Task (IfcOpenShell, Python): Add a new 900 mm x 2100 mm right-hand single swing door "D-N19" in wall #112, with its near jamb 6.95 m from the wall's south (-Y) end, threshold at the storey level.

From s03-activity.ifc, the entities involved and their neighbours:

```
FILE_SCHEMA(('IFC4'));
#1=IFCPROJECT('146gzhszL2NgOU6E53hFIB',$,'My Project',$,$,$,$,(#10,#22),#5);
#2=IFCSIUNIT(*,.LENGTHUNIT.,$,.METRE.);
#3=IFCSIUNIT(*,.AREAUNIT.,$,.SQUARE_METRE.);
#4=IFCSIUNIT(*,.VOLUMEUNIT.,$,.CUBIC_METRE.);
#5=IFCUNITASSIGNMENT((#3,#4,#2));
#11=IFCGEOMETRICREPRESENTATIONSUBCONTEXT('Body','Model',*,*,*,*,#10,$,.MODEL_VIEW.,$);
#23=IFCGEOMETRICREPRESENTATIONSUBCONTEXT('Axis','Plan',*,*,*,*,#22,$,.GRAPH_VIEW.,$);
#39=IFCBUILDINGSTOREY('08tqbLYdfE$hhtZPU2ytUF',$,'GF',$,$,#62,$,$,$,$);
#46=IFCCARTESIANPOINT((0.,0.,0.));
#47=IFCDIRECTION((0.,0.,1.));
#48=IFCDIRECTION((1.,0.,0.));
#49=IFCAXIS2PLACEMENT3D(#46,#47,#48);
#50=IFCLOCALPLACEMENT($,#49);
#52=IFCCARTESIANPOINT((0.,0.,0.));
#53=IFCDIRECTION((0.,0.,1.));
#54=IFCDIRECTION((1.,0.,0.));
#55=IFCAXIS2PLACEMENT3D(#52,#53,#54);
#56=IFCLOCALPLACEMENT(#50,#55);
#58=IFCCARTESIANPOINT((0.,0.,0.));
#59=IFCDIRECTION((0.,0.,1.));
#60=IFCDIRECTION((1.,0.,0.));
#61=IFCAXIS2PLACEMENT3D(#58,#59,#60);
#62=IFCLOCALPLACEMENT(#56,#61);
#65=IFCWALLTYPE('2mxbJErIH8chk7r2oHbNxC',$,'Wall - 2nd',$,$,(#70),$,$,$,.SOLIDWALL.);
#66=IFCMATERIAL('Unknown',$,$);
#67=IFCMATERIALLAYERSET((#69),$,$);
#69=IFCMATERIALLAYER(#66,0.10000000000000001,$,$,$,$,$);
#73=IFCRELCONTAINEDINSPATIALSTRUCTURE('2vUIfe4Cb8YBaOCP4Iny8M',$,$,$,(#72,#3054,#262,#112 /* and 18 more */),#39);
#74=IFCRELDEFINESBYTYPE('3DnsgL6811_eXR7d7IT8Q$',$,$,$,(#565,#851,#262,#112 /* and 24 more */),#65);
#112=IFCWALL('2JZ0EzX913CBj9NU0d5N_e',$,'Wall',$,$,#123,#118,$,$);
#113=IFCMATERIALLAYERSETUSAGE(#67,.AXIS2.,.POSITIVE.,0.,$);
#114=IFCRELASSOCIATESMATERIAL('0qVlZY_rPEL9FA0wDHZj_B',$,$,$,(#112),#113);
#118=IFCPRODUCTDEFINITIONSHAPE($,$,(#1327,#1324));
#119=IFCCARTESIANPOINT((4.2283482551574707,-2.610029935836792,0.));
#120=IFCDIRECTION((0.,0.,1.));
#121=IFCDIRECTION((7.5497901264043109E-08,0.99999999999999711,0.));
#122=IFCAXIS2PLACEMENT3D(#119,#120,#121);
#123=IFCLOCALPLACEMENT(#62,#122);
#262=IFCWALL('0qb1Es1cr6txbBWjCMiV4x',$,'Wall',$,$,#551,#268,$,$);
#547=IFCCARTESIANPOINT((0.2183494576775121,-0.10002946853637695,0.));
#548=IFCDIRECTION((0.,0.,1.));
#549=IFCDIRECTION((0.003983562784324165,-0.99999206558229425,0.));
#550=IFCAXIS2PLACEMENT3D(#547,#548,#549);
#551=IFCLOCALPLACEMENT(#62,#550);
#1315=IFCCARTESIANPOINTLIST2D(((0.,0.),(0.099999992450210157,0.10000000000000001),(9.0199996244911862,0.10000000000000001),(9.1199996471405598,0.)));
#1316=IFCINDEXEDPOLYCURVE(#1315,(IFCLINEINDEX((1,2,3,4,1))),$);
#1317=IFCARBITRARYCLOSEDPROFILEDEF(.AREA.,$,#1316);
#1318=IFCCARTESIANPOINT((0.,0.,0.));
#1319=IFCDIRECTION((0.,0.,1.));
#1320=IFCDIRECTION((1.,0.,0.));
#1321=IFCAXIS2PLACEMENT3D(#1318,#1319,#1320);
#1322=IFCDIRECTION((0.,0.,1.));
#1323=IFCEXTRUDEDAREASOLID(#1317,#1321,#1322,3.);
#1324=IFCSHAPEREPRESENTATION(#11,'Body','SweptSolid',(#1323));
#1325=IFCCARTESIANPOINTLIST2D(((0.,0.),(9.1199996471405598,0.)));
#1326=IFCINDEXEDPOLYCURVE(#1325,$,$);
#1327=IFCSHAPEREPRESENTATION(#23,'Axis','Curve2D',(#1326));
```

```python
import numpy as np
import ifcopenshell
import ifcopenshell.api.feature
import ifcopenshell.api.geometry
import ifcopenshell.api.root
import ifcopenshell.api.spatial
import ifcopenshell.geom
import ifcopenshell.util.element
import ifcopenshell.util.placement
import ifcopenshell.util.representation
import ifcopenshell.util.shape
import ifcopenshell.util.unit

model = ifcopenshell.open("s03-activity.ifc")
unit_scale = ifcopenshell.util.unit.calculate_unit_scale(model)
settings = ifcopenshell.geom.settings()


def volume(element):
    """Net volume in cubic metres, openings subtracted."""
    shape = ifcopenshell.geom.create_shape(settings, element)
    return ifcopenshell.util.shape.get_volume(shape.geometry)


wall = model.by_guid("2JZ0EzX913CBj9NU0d5N_e")
storey = ifcopenshell.util.element.get_container(wall, ifc_class="IfcBuildingStorey")
context = ifcopenshell.util.representation.get_context(model, "Model", "Body", "MODEL_VIEW")
before = volume(wall)

width, height, from_end, sill = 0.9, 2.1, 6.95, 0.0  # metres

# The wall runs along its own X axis, and the end named is its -X end.
wall_shape = ifcopenshell.geom.create_shape(settings, wall)
x, y, z = ifcopenshell.util.shape.get_vertices(wall_shape.geometry).T
start = x.min() + from_end
face, thickness = float(y.min()), float(y.max() - y.min())
wall_matrix = ifcopenshell.util.placement.get_local_placement(wall.ObjectPlacement)
level = ifcopenshell.util.placement.get_local_placement(storey.ObjectPlacement)[2, 3]


def in_wall(x, y):
    """Placement at x, y metres in the wall's axes, at sill height."""
    matrix = wall_matrix.copy()
    matrix[:, 3] = wall_matrix @ np.array([x / unit_scale, y / unit_scale, 0.0, 1.0])
    matrix[2, 3] = level + sill / unit_scale
    return matrix


# Opening: a box that overshoots both wall faces by 50 mm.
opening = ifcopenshell.api.root.create_entity(model, ifc_class="IfcOpeningElement", predefined_type="OPENING")
box = ifcopenshell.api.geometry.add_wall_representation(
    model, context=context, length=width, height=height, thickness=thickness + 0.1
)
ifcopenshell.api.geometry.assign_representation(model, product=opening, representation=box)
ifcopenshell.api.geometry.edit_object_placement(model, product=opening, matrix=in_wall(start, face - 0.05), is_si=False)
ifcopenshell.api.feature.add_feature(model, feature=opening, element=wall)

door = ifcopenshell.api.root.create_entity(model, ifc_class="IfcDoor", name="D-N19", predefined_type="DOOR")
door.OverallWidth, door.OverallHeight = width / unit_scale, height / unit_scale
door.OperationType = "SINGLE_SWING_RIGHT"
body = ifcopenshell.api.geometry.add_door_representation(
    model,
    context=context,
    overall_width=door.OverallWidth,
    overall_height=door.OverallHeight,
    operation_type="SINGLE_SWING_RIGHT",
    lining_properties={"LiningDepth": thickness / unit_scale, "ThresholdDepth": thickness / unit_scale},
)
ifcopenshell.api.geometry.assign_representation(model, product=door, representation=body)
ifcopenshell.api.spatial.assign_container(model, products=[door], relating_structure=storey)
ifcopenshell.api.feature.add_filling(model, opening=opening, element=door)

# The lining spans the wall, so the door starts at the wall face.
ifcopenshell.api.geometry.edit_object_placement(model, product=door, matrix=in_wall(start, face), is_si=False)

after = volume(wall)

print(f"wall volume {before:.3f} -> {after:.3f} m3")

model.write("s03-activity_edited.ifc")
```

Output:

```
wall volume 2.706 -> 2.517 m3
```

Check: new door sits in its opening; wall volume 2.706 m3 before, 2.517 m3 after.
